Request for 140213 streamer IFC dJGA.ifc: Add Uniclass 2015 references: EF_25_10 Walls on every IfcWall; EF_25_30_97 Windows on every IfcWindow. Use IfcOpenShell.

First a look at what the model holds.

```python
import ifcopenshell

model = ifcopenshell.open("140213 streamer IFC dJGA.ifc")
print(model.schema)
print("classifications:", [c.Name for c in model.by_type("IfcClassification")])
for ifc_class in ("IfcDoor", "IfcRoof", "IfcStair", "IfcWall", "IfcWindow"):
    print(ifc_class, len(model.by_type(ifc_class)))
```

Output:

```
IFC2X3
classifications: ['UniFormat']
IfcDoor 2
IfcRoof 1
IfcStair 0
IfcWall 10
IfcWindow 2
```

```python
import ifcopenshell
import ifcopenshell.api.classification

model = ifcopenshell.open("140213 streamer IFC dJGA.ifc")

# IFC2X3 requires Source and Edition and has no link from the project to the system.
system = model.create_entity("IfcClassification", Source="NBS", Edition="2015", Name="Uniclass 2015")

codes = {
    "IfcWall": ("EF_25_10", "Walls"),
    "IfcWindow": ("EF_25_30_97", "Windows"),
}
for ifc_class, (code, name) in codes.items():
    products = model.by_type(ifc_class)
    ifcopenshell.api.classification.add_reference(
        model, products=products, classification=system, identification=code, name=name
    )
    print(code, len(products))

model.write("140213 streamer IFC dJGA-out.ifc")
```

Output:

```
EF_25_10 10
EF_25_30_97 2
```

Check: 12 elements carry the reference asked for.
